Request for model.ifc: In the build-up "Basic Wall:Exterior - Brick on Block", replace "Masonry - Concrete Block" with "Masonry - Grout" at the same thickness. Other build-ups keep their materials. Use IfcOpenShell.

First a look at what the model holds.

```python
import ifcopenshell
import ifcopenshell.util.element

model = ifcopenshell.open("model.ifc")
print(model.schema)
for layer_set in model.by_type("IfcMaterialLayerSet"):
    if layer_set.LayerSetName == "Basic Wall:Exterior - Brick on Block":
        for layer in layer_set.MaterialLayers:
            print(layer.id(), layer.Material and layer.Material.Name, layer.LayerThickness, sep=" | ")
        print(len(ifcopenshell.util.element.get_elements_by_material(model, layer_set)), "elements and types use it")
print(sorted(m.Name for m in model.by_type("IfcMaterial") if m.Name)[:60])
```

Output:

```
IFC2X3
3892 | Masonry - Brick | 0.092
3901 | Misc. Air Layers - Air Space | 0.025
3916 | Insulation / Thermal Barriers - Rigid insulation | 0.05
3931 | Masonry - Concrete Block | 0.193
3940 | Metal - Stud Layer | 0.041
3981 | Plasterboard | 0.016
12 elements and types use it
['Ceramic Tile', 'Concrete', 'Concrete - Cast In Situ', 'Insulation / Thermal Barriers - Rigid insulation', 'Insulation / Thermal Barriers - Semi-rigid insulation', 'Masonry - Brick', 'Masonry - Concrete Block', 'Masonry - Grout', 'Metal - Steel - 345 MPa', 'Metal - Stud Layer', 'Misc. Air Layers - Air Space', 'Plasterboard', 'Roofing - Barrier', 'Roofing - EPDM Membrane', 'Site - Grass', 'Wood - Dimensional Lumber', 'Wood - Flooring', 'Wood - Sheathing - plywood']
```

```python
import ifcopenshell
import ifcopenshell.api.material

model = ifcopenshell.open("model.ifc")

layer_set = next(s for s in model.by_type("IfcMaterialLayerSet") if s.LayerSetName == "Basic Wall:Exterior - Brick on Block")
layer = next(l for l in layer_set.MaterialLayers if l.Material and l.Material.Name == "Masonry - Concrete Block")
material = next(m for m in model.by_type("IfcMaterial") if m.Name == "Masonry - Grout")

# Point this one layer at the other material; renaming the old one would change it everywhere.
ifcopenshell.api.material.edit_layer(model, layer=layer, attributes={}, material=material)

print([l.Material.Name if l.Material else None for l in layer_set.MaterialLayers])

model.write("model_v2.ifc")
```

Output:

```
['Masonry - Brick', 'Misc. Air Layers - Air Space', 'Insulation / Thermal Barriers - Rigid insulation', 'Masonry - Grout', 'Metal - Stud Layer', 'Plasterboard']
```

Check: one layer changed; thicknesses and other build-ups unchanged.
